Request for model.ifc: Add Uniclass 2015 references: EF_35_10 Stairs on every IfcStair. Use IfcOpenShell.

First a look at what the model holds.

```python
import ifcopenshell

model = ifcopenshell.open("model.ifc")
print(model.schema)
print("classifications:", [c.Name for c in model.by_type("IfcClassification")])
for ifc_class in ("IfcDoor", "IfcRoof", "IfcStair", "IfcWall", "IfcWindow"):
    print(ifc_class, len(model.by_type(ifc_class)))
```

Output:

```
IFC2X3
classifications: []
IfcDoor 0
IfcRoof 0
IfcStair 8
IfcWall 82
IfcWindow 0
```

```python
import ifcopenshell
import ifcopenshell.api.classification

model = ifcopenshell.open("model.ifc")

# IFC2X3 requires Source and Edition and has no link from the project to the system.
system = model.create_entity("IfcClassification", Source="NBS", Edition="2015", Name="Uniclass 2015")

codes = {
    "IfcStair": ("EF_35_10", "Stairs"),
}
for ifc_class, (code, name) in codes.items():
    products = model.by_type(ifc_class)
    ifcopenshell.api.classification.add_reference(
        model, products=products, classification=system, identification=code, name=name
    )
    print(code, len(products))

model.write("model_edited.ifc")
```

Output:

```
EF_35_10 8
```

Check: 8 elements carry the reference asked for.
